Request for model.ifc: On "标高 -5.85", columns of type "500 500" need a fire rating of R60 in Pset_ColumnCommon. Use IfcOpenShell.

First a look at what the model holds.

```python
import ifcopenshell
import ifcopenshell.util.element

model = ifcopenshell.open("model.ifc")
print(model.schema)
storey = next(s for s in model.by_type("IfcBuildingStorey") if s.Name == "标高 -5.85")
columns = [e for e in ifcopenshell.util.element.get_decomposition(storey) if e.is_a("IfcColumn")]
seen = {}
for e in columns:
    element_type = ifcopenshell.util.element.get_type(e)
    key = (element_type.Name if element_type != e and element_type else None, ifcopenshell.util.element.get_pset(e, "Pset_ColumnCommon", "FireRating"))
    seen[key] = seen.get(key, 0) + 1
for (name, value), count in sorted(seen.items(), key=str):
    print(count, "x", name, "|", value)
```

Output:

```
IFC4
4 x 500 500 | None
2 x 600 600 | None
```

```python
import ifcopenshell
import ifcopenshell.api.pset
import ifcopenshell.util.element

model = ifcopenshell.open("model.ifc")

storey = next(s for s in model.by_type("IfcBuildingStorey") if s.Name == "标高 -5.85")
columns = [e for e in ifcopenshell.util.element.get_decomposition(storey) if e.is_a("IfcColumn")]

count = 0
for e in columns:
    element_type = ifcopenshell.util.element.get_type(e)
    if element_type in (None, e) or element_type.Name != "500 500":
        continue
    # add_pset returns the element's existing set when there is one.
    pset = ifcopenshell.api.pset.add_pset(model, product=e, name="Pset_ColumnCommon")
    ifcopenshell.api.pset.edit_pset(model, pset=pset, properties={"FireRating": "R60"})
    count += 1

print(count, "columns updated")

model.write("model_v2.ifc")
```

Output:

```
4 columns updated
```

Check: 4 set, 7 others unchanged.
